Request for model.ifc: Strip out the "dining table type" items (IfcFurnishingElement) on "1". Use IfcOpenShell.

First a look at what the model holds.

```python
import ifcopenshell
import ifcopenshell.util.element

model = ifcopenshell.open("model.ifc")
print(model.schema)
storey = next(s for s in model.by_type("IfcBuildingStorey") if s.Name == "1")
furniture = [e for e in ifcopenshell.util.element.get_decomposition(storey) if e.is_a("IfcFurnishingElement")]
seen = {}
for e in furniture:
    element_type = ifcopenshell.util.element.get_type(e)
    name = element_type.Name if element_type not in (None, e) else None
    seen[name] = seen.get(name, 0) + 1
for name, count in sorted(seen.items(), key=str):
    print(count, "x", name)
```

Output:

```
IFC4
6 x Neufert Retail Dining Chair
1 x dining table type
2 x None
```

```python
import ifcopenshell
import ifcopenshell.api.root
import ifcopenshell.util.element

model = ifcopenshell.open("model.ifc")

storey = next(s for s in model.by_type("IfcBuildingStorey") if s.Name == "1")
furniture = [e for e in ifcopenshell.util.element.get_decomposition(storey) if e.is_a("IfcFurnishingElement")]
targets = [e for e in furniture if (t := ifcopenshell.util.element.get_type(e)) not in (None, e) and t.Name == "dining table type"]

for e in targets:
    ifcopenshell.api.root.remove_product(model, product=e)
print(len(targets), "removed")

model.write("model_updated.ifc")
```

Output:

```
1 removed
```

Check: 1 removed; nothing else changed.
